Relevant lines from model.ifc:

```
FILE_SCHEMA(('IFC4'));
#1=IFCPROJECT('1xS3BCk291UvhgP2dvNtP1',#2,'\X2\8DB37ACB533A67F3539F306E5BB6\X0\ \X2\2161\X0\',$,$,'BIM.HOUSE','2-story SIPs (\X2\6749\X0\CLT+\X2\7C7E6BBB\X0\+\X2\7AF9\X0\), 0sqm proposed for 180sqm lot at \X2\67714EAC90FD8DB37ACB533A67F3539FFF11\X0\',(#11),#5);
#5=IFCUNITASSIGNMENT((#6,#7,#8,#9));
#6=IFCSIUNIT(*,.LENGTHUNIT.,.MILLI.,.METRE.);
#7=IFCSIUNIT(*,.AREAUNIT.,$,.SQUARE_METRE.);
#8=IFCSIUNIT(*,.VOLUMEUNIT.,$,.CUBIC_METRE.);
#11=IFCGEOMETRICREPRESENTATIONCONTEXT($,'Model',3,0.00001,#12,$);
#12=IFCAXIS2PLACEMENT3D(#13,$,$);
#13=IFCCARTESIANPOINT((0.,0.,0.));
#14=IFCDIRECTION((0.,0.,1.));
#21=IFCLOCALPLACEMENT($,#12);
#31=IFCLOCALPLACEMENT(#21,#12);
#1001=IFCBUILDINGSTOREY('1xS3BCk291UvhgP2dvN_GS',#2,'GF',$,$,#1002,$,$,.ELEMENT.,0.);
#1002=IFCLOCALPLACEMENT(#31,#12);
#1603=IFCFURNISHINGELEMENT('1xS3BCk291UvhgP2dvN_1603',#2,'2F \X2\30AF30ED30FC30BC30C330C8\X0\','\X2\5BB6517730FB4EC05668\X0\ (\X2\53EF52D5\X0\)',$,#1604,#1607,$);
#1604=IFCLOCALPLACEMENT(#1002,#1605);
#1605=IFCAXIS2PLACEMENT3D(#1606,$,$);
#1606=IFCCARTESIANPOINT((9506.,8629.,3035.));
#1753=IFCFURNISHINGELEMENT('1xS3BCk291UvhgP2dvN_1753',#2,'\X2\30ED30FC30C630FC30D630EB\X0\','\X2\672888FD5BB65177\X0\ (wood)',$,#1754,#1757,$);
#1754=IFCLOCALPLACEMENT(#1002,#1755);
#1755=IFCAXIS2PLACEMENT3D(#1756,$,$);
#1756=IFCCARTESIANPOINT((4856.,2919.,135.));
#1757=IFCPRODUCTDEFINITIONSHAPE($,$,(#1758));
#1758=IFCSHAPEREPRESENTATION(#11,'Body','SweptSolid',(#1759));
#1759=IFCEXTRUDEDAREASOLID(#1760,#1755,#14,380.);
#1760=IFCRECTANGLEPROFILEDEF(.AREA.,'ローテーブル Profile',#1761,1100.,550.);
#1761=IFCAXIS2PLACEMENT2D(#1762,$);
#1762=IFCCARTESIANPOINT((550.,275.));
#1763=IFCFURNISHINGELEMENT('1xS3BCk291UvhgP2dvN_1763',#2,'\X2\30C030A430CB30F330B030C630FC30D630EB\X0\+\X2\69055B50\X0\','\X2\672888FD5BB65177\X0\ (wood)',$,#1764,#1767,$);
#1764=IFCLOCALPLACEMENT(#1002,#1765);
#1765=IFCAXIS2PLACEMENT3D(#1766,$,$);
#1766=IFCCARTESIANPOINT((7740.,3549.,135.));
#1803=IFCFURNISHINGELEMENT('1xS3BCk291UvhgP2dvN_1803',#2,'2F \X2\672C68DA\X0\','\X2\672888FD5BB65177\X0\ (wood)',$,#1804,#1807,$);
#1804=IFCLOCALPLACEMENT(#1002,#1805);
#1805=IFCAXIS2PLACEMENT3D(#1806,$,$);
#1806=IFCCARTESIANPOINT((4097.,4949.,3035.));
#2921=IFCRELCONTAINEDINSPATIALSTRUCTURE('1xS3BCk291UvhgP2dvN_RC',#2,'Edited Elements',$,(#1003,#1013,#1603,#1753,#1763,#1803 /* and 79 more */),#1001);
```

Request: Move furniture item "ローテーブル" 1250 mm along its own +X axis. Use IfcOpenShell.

```python
import ifcopenshell
import ifcopenshell.api.geometry
import ifcopenshell.util.placement

model = ifcopenshell.open("model.ifc")

item = model.by_guid("1xS3BCk291UvhgP2dvN_1753")
matrix = ifcopenshell.util.placement.get_local_placement(item.ObjectPlacement)
matrix[:3, 3] += matrix[:3, 0] * 1250.0
ifcopenshell.api.geometry.edit_object_placement(model, product=item, matrix=matrix, is_si=False)

print(ifcopenshell.util.placement.get_local_placement(item.ObjectPlacement).round(3) + 0.0)

model.write("model_edited.ifc")
```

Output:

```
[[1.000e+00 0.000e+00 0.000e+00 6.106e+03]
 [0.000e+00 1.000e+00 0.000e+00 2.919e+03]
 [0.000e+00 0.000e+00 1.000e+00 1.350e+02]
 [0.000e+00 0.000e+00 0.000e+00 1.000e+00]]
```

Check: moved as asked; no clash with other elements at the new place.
